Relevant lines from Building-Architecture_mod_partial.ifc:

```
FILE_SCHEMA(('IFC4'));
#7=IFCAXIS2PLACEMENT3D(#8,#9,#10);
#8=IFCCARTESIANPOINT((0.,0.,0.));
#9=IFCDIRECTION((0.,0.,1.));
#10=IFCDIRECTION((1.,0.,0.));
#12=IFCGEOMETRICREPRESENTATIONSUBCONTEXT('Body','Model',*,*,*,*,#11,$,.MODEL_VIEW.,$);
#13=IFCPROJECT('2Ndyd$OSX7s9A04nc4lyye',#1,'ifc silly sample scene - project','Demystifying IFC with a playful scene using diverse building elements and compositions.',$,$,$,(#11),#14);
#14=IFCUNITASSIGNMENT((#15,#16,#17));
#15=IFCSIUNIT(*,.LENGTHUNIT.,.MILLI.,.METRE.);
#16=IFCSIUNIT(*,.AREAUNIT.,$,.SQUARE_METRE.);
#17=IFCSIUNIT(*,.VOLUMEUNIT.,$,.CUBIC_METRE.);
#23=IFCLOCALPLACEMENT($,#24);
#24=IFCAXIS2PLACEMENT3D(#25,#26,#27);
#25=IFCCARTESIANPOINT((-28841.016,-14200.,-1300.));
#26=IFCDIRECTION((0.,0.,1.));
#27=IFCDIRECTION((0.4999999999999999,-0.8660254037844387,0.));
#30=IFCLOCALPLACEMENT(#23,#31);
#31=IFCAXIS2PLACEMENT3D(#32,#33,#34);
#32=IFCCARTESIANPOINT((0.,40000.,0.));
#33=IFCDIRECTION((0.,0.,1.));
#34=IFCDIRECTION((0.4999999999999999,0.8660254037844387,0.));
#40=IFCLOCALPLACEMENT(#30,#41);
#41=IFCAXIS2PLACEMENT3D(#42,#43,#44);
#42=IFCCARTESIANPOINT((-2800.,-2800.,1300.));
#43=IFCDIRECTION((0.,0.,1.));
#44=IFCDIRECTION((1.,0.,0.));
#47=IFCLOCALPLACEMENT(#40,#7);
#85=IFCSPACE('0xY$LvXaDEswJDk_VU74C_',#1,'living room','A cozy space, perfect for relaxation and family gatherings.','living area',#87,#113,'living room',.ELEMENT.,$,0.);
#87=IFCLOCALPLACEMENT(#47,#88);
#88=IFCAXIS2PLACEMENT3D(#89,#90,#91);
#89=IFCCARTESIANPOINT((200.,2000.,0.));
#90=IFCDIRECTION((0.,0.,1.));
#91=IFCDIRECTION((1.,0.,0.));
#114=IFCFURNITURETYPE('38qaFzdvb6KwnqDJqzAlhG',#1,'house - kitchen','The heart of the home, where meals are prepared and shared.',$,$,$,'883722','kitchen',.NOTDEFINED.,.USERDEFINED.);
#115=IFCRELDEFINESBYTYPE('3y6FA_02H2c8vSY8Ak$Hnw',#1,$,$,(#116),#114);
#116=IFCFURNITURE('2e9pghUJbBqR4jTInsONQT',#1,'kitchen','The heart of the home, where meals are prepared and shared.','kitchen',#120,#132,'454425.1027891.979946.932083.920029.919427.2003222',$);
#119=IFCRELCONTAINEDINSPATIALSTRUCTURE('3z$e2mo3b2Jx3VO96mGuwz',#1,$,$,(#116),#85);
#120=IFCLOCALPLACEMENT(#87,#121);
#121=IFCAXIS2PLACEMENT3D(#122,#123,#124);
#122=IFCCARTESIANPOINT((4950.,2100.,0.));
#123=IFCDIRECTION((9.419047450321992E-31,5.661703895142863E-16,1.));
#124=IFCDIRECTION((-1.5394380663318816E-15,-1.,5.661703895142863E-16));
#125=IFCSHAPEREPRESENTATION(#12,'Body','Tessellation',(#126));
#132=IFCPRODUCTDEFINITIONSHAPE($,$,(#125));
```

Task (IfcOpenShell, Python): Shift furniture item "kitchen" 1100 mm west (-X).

```python
import ifcopenshell
import ifcopenshell.api.geometry
import ifcopenshell.util.placement
import ifcopenshell.util.unit

model = ifcopenshell.open("Building-Architecture_mod_partial.ifc")
unit_scale = ifcopenshell.util.unit.calculate_unit_scale(model)

item = model.by_guid("2e9pghUJbBqR4jTInsONQT")
matrix = ifcopenshell.util.placement.get_local_placement(item.ObjectPlacement)
matrix[0, 3] -= 1.1 / unit_scale
ifcopenshell.api.geometry.edit_object_placement(model, product=item, matrix=matrix, is_si=False)

print(ifcopenshell.util.placement.get_local_placement(item.ObjectPlacement).round(3) + 0.0)

model.write("Building-Architecture_mod_partial_rev.ifc")
```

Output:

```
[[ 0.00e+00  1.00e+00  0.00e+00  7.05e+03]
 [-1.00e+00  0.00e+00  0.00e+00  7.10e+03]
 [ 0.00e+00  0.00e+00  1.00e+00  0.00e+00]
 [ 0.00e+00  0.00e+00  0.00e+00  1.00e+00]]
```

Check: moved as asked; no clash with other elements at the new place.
